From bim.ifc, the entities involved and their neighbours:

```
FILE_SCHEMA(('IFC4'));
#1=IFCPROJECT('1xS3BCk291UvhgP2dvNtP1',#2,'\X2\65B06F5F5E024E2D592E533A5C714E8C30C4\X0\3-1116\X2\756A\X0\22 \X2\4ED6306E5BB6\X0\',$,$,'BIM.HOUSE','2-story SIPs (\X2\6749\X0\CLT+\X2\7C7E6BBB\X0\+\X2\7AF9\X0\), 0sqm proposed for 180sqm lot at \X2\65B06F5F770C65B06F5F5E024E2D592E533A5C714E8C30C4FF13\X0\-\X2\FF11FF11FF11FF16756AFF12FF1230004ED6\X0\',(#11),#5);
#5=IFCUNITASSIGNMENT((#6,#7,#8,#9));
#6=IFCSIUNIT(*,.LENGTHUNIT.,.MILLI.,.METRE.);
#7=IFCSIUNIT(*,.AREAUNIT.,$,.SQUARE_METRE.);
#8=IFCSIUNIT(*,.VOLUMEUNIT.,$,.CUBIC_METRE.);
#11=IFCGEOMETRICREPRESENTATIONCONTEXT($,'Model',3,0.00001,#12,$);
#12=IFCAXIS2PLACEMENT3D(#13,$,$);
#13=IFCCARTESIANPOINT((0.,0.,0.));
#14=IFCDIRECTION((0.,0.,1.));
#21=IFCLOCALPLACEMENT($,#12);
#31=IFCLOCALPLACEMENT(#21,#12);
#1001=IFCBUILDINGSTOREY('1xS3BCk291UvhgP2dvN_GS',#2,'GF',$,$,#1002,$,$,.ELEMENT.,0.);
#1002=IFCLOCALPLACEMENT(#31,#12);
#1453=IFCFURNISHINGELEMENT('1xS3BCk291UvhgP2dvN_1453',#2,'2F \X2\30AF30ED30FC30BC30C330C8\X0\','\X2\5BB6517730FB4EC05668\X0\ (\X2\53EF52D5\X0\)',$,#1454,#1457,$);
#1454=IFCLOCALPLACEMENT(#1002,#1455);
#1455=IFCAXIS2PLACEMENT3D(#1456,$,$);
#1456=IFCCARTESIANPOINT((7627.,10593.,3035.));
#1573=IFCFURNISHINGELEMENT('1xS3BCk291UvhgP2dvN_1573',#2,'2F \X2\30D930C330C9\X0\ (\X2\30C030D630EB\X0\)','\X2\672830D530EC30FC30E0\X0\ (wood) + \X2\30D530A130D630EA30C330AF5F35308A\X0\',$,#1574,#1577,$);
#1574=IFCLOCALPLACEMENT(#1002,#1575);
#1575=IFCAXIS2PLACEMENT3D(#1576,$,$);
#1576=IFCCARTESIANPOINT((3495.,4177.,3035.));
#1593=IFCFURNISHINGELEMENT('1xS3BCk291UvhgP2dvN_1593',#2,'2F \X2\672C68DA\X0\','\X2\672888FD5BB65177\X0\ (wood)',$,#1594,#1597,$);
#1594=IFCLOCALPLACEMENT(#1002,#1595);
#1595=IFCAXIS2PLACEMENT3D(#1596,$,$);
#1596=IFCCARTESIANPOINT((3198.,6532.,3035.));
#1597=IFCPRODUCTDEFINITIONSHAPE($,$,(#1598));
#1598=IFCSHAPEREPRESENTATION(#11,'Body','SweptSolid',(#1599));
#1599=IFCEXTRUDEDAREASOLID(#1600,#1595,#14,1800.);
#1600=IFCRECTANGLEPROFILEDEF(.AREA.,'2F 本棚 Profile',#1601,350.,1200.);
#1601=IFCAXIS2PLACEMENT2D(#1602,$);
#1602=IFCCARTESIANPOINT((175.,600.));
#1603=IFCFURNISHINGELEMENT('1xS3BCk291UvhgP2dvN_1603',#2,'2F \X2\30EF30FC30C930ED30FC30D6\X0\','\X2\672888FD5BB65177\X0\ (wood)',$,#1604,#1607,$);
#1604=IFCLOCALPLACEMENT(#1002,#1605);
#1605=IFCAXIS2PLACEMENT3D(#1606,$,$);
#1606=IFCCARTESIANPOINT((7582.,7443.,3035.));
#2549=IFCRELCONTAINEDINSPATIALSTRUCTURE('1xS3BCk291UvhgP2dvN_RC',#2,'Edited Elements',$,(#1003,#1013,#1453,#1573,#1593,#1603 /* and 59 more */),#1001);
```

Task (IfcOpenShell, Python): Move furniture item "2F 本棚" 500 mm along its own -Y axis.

```python
import ifcopenshell
import ifcopenshell.api.geometry
import ifcopenshell.util.placement
import ifcopenshell.util.unit

model = ifcopenshell.open("bim.ifc")
unit_scale = ifcopenshell.util.unit.calculate_unit_scale(model)

item = model.by_guid("1xS3BCk291UvhgP2dvN_1593")
matrix = ifcopenshell.util.placement.get_local_placement(item.ObjectPlacement)
matrix[:3, 3] -= matrix[:3, 1] * 0.5 / unit_scale
ifcopenshell.api.geometry.edit_object_placement(model, product=item, matrix=matrix, is_si=False)

print(ifcopenshell.util.placement.get_local_placement(item.ObjectPlacement).round(3) + 0.0)

model.write("bim-out.ifc")
```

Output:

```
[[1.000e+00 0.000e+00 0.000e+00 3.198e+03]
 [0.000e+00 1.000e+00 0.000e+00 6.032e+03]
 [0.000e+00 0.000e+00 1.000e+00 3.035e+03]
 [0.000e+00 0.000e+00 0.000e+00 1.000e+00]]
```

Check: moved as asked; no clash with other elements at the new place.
